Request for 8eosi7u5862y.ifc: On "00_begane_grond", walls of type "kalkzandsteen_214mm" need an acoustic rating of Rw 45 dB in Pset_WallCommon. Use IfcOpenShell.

First a look at what the model holds.

```python
import ifcopenshell
import ifcopenshell.util.element

model = ifcopenshell.open("8eosi7u5862y.ifc")
print(model.schema)
storey = next(s for s in model.by_type("IfcBuildingStorey") if s.Name == "00_begane_grond")
walls = [e for e in ifcopenshell.util.element.get_decomposition(storey) if e.is_a("IfcWall")]
seen = {}
for e in walls:
    element_type = ifcopenshell.util.element.get_type(e)
    key = (element_type.Name if element_type != e and element_type else None, ifcopenshell.util.element.get_pset(e, "Pset_WallCommon", "AcousticRating"))
    seen[key] = seen.get(key, 0) + 1
for (name, value), count in sorted(seen.items(), key=str):
    print(count, "x", name, "|", value)
```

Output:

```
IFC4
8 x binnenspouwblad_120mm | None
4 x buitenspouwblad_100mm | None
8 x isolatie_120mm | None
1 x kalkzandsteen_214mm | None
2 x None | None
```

```python
import ifcopenshell
import ifcopenshell.api.pset
import ifcopenshell.util.element

model = ifcopenshell.open("8eosi7u5862y.ifc")

storey = next(s for s in model.by_type("IfcBuildingStorey") if s.Name == "00_begane_grond")
walls = [e for e in ifcopenshell.util.element.get_decomposition(storey) if e.is_a("IfcWall")]

count = 0
for e in walls:
    element_type = ifcopenshell.util.element.get_type(e)
    if element_type in (None, e) or element_type.Name != "kalkzandsteen_214mm":
        continue
    # add_pset returns the element's existing set when there is one.
    pset = ifcopenshell.api.pset.add_pset(model, product=e, name="Pset_WallCommon")
    ifcopenshell.api.pset.edit_pset(model, pset=pset, properties={"AcousticRating": "Rw 45 dB"})
    count += 1

print(count, "walls updated")

model.write("8eosi7u5862y_rev.ifc")
```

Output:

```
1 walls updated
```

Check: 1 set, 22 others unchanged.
